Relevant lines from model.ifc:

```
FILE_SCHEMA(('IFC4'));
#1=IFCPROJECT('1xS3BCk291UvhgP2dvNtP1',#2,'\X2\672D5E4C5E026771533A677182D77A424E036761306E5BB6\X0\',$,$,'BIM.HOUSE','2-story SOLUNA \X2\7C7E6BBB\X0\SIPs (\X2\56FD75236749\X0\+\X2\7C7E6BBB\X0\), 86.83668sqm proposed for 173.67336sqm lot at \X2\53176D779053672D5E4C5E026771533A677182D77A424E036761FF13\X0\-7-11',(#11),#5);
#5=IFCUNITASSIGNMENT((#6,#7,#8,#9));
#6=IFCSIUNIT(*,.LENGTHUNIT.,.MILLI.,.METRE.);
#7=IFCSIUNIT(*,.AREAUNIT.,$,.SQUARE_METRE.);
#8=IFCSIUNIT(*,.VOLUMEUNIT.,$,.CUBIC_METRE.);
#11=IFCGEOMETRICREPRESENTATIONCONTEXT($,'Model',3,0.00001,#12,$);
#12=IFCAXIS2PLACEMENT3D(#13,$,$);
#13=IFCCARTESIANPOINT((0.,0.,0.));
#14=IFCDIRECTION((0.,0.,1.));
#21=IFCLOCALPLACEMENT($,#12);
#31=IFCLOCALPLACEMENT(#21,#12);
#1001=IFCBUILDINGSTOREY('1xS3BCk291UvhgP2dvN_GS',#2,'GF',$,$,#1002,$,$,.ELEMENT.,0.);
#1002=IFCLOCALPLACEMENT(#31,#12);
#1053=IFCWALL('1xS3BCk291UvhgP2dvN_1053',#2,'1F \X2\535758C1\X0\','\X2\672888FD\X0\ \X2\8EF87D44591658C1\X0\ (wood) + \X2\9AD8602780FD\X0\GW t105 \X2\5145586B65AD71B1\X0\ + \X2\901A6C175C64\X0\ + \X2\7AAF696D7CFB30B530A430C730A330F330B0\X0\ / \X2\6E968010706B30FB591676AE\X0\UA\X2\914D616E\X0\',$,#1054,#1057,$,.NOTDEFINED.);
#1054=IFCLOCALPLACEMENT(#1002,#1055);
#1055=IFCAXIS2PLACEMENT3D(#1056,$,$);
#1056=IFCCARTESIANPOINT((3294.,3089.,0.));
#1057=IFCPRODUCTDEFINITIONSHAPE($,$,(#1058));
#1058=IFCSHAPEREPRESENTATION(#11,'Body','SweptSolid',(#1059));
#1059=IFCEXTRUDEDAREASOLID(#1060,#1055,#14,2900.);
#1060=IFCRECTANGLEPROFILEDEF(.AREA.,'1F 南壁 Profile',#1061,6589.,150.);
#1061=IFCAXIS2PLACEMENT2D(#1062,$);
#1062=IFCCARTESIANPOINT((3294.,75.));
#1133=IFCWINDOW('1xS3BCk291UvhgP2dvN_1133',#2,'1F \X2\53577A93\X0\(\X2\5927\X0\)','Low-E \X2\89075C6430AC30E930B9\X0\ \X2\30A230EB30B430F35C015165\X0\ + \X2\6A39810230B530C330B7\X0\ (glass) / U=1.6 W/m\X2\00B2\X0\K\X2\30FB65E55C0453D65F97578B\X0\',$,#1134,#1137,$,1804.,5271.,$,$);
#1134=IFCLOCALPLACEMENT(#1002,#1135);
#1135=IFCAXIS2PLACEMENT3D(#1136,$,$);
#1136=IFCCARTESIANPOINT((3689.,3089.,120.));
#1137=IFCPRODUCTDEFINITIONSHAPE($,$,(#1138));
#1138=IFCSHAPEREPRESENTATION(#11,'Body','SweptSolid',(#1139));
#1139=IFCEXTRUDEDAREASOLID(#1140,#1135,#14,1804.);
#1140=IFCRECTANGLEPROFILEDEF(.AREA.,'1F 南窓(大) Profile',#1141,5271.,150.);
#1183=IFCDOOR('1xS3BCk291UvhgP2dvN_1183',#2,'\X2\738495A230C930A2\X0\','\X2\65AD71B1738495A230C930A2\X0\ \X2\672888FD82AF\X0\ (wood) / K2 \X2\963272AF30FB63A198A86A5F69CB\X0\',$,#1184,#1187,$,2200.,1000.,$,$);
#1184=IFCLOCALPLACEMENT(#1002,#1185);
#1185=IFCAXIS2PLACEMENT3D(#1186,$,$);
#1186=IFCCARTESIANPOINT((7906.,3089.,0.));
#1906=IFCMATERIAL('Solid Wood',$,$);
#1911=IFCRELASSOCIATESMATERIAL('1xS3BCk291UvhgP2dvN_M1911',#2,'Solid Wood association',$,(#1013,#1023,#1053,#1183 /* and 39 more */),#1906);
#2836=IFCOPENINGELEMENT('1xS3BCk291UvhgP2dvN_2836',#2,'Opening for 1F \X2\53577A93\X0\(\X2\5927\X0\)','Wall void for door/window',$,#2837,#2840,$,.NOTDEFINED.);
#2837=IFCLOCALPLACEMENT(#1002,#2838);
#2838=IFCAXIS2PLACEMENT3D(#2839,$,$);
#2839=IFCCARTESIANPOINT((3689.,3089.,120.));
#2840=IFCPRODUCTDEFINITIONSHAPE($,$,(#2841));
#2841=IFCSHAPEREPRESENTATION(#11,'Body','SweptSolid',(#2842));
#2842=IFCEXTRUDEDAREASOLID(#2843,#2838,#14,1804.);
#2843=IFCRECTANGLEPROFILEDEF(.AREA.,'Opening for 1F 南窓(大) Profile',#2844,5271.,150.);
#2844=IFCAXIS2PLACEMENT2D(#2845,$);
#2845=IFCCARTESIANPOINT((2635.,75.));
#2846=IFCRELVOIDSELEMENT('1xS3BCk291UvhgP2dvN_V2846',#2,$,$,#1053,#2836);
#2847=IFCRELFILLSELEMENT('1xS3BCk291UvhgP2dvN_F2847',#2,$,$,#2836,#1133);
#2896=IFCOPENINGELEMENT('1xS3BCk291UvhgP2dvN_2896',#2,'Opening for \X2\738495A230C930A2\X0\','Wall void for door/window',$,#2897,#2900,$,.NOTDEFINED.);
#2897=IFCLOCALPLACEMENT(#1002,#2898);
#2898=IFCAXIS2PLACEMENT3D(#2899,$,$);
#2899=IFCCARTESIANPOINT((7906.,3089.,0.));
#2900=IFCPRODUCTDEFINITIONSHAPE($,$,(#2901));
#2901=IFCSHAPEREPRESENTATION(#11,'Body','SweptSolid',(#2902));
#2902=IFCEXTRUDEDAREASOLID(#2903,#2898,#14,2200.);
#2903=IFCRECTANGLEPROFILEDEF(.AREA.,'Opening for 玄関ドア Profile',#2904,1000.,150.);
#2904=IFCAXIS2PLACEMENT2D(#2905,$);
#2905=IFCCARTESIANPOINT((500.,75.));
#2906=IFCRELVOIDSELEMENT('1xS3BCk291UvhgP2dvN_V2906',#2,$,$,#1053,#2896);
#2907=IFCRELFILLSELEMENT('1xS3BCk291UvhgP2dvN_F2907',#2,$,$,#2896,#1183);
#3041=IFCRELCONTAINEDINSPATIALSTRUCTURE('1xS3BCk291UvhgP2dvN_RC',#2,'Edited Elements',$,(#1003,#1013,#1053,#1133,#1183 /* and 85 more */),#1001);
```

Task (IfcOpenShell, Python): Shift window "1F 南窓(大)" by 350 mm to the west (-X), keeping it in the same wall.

```python
import ifcopenshell
import ifcopenshell.api.geometry
import ifcopenshell.util.placement
import ifcopenshell.util.unit

model = ifcopenshell.open("model.ifc")
unit_scale = ifcopenshell.util.unit.calculate_unit_scale(model)

window = model.by_id(1133)
opening = window.FillsVoids[0].RelatingOpeningElement
wall = opening.VoidsElements[0].RelatingBuildingElement

wall_matrix = ifcopenshell.util.placement.get_local_placement(wall.ObjectPlacement)
shift = wall_matrix[:3, 0] * -0.35 / unit_scale
before = ifcopenshell.util.placement.get_local_placement(window.ObjectPlacement)[:3, 3].copy()

# The window is not placed relative to its opening, so move both.
for product in (opening, window):
    matrix = ifcopenshell.util.placement.get_local_placement(product.ObjectPlacement)
    matrix[:3, 3] += shift
    ifcopenshell.api.geometry.edit_object_placement(model, product=product, matrix=matrix, is_si=False)

after = ifcopenshell.util.placement.get_local_placement(window.ObjectPlacement)[:3, 3]
print("window moved by", (after - before).round(3) + 0.0)

model.write("model_edited.ifc")
```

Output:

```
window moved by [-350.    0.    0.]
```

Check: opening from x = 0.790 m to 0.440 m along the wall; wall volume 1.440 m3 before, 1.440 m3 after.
